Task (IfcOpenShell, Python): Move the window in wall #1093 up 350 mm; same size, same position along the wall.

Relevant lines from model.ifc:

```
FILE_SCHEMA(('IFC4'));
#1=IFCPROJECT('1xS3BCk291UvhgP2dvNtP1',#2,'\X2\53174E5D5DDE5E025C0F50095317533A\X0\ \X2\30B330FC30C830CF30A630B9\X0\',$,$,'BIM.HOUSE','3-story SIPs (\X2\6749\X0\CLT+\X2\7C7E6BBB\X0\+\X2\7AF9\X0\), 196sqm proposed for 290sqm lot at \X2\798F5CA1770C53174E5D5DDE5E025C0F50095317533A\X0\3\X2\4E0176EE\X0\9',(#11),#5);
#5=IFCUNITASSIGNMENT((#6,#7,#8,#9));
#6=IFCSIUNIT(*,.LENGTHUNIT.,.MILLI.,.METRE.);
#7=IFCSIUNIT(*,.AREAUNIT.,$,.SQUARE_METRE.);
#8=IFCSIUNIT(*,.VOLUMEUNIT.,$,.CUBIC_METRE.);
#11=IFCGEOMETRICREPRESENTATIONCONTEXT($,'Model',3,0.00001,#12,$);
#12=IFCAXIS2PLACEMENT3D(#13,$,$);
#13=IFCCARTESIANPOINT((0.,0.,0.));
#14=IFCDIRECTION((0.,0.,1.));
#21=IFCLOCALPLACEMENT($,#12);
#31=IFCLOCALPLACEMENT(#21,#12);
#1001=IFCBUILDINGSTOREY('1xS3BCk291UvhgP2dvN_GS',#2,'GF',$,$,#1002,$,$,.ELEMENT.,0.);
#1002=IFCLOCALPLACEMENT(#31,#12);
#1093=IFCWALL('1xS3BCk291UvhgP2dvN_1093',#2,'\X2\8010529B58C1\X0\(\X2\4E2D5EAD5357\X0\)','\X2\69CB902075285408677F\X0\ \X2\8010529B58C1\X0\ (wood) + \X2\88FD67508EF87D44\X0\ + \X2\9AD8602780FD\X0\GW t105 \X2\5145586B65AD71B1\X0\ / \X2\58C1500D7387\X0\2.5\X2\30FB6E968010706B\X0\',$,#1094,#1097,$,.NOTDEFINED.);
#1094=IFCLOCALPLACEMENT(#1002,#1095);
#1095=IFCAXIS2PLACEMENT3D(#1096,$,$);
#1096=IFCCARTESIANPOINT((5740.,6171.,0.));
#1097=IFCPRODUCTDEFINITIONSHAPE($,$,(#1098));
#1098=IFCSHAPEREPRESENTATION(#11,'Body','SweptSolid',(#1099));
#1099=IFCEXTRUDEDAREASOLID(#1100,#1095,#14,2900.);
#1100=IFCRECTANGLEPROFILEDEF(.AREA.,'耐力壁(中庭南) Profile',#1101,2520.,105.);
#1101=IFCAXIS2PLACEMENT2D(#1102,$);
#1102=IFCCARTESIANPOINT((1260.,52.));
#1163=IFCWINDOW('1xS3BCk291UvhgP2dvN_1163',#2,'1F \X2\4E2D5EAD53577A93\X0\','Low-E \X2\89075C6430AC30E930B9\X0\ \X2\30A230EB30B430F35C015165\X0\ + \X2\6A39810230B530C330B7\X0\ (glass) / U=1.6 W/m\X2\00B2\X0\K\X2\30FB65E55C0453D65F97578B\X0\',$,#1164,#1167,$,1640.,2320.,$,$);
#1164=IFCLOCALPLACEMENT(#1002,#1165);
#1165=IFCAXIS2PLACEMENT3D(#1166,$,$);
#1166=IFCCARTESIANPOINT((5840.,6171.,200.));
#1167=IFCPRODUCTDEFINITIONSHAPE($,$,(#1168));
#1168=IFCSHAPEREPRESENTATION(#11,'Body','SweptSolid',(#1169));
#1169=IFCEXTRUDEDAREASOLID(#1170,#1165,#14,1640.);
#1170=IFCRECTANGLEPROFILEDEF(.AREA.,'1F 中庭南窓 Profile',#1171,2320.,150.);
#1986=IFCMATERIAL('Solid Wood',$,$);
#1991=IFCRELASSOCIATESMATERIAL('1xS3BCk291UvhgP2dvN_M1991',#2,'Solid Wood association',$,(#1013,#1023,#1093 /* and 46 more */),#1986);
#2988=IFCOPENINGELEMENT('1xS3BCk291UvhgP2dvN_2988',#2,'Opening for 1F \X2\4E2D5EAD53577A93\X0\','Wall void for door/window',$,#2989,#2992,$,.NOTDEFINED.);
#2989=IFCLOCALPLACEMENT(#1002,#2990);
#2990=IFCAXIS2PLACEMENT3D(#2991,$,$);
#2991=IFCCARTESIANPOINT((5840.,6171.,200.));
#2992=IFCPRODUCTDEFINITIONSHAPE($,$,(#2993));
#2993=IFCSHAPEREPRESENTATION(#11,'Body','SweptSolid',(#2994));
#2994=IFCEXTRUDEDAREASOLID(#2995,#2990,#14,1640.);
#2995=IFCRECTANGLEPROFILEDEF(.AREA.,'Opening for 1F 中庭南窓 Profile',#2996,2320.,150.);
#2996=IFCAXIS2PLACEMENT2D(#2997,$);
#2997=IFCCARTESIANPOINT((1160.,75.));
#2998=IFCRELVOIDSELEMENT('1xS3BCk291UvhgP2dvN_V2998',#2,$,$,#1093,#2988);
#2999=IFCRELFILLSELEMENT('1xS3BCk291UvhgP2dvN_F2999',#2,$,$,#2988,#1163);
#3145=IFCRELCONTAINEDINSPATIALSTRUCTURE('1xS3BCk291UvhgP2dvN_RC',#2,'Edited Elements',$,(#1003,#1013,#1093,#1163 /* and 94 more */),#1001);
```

```python
import numpy as np
import ifcopenshell
import ifcopenshell.api.geometry
import ifcopenshell.util.placement
import ifcopenshell.util.unit

model = ifcopenshell.open("model.ifc")
unit_scale = ifcopenshell.util.unit.calculate_unit_scale(model)

window = model.by_guid("1xS3BCk291UvhgP2dvN_1163")
opening = window.FillsVoids[0].RelatingOpeningElement
dz = 0.35 / unit_scale

shift = np.array([0.0, 0.0, dz])
# The window is not placed relative to its opening, so move both.
for product in (opening, window):
    matrix = ifcopenshell.util.placement.get_local_placement(product.ObjectPlacement)
    matrix[:3, 3] += shift
    ifcopenshell.api.geometry.edit_object_placement(model, product=product, matrix=matrix, is_si=False)

print(f"moved by {dz * unit_scale:+.3f} m")

model.write("model_v2.ifc")
```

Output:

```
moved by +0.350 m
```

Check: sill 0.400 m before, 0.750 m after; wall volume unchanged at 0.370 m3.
